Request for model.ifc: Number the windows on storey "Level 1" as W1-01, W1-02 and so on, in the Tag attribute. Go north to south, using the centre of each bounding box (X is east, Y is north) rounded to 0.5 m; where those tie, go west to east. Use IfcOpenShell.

First a look at what the model holds.

```python
import ifcopenshell
import ifcopenshell.util.element
import ifcopenshell.util.placement

model = ifcopenshell.open("model.ifc")
print(model.schema)
storey = next(s for s in model.by_type("IfcBuildingStorey") if s.Name == "Level 1")
windows = [e for e in ifcopenshell.util.element.get_decomposition(storey) if e.is_a("IfcWindow")]
for e in sorted(windows, key=lambda e: e.id()):
    origin = ifcopenshell.util.placement.get_local_placement(e.ObjectPlacement)[:3, 3]
    print(e.id(), e.Tag, e.Name, origin.round(2) + 0.0, sep=" | ")
```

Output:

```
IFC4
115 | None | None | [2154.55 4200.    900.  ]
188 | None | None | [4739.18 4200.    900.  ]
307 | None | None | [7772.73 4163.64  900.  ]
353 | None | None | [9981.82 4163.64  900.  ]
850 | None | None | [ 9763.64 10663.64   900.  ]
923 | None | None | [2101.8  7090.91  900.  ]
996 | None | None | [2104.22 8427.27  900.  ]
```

```python
import ifcopenshell
import ifcopenshell.geom
import ifcopenshell.util.element
import ifcopenshell.util.shape

model = ifcopenshell.open("model.ifc")
settings = ifcopenshell.geom.settings()
settings.set("use-world-coords", True)


def centre(element):
    shape = ifcopenshell.geom.create_shape(settings, element)
    return ifcopenshell.util.shape.get_bbox_centroid(shape.geometry)


storey = next(s for s in model.by_type("IfcBuildingStorey") if s.Name == "Level 1")
windows = [e for e in ifcopenshell.util.element.get_decomposition(storey) if e.is_a("IfcWindow")]

# Insertion points can sit at a corner or the storey origin, so sort by the geometry (in metres).
centres = {e: centre(e) for e in windows}
windows.sort(key=lambda e: (-round(centres[e][1] / 0.5), centres[e][0]))

for i, e in enumerate(windows, start=1):
    number = f"W1-{i:02d}"
    e.Tag = number
    print(e.id(), number)

model.write("model_edited.ifc")
```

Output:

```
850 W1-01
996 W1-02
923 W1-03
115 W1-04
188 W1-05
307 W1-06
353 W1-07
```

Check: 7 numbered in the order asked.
